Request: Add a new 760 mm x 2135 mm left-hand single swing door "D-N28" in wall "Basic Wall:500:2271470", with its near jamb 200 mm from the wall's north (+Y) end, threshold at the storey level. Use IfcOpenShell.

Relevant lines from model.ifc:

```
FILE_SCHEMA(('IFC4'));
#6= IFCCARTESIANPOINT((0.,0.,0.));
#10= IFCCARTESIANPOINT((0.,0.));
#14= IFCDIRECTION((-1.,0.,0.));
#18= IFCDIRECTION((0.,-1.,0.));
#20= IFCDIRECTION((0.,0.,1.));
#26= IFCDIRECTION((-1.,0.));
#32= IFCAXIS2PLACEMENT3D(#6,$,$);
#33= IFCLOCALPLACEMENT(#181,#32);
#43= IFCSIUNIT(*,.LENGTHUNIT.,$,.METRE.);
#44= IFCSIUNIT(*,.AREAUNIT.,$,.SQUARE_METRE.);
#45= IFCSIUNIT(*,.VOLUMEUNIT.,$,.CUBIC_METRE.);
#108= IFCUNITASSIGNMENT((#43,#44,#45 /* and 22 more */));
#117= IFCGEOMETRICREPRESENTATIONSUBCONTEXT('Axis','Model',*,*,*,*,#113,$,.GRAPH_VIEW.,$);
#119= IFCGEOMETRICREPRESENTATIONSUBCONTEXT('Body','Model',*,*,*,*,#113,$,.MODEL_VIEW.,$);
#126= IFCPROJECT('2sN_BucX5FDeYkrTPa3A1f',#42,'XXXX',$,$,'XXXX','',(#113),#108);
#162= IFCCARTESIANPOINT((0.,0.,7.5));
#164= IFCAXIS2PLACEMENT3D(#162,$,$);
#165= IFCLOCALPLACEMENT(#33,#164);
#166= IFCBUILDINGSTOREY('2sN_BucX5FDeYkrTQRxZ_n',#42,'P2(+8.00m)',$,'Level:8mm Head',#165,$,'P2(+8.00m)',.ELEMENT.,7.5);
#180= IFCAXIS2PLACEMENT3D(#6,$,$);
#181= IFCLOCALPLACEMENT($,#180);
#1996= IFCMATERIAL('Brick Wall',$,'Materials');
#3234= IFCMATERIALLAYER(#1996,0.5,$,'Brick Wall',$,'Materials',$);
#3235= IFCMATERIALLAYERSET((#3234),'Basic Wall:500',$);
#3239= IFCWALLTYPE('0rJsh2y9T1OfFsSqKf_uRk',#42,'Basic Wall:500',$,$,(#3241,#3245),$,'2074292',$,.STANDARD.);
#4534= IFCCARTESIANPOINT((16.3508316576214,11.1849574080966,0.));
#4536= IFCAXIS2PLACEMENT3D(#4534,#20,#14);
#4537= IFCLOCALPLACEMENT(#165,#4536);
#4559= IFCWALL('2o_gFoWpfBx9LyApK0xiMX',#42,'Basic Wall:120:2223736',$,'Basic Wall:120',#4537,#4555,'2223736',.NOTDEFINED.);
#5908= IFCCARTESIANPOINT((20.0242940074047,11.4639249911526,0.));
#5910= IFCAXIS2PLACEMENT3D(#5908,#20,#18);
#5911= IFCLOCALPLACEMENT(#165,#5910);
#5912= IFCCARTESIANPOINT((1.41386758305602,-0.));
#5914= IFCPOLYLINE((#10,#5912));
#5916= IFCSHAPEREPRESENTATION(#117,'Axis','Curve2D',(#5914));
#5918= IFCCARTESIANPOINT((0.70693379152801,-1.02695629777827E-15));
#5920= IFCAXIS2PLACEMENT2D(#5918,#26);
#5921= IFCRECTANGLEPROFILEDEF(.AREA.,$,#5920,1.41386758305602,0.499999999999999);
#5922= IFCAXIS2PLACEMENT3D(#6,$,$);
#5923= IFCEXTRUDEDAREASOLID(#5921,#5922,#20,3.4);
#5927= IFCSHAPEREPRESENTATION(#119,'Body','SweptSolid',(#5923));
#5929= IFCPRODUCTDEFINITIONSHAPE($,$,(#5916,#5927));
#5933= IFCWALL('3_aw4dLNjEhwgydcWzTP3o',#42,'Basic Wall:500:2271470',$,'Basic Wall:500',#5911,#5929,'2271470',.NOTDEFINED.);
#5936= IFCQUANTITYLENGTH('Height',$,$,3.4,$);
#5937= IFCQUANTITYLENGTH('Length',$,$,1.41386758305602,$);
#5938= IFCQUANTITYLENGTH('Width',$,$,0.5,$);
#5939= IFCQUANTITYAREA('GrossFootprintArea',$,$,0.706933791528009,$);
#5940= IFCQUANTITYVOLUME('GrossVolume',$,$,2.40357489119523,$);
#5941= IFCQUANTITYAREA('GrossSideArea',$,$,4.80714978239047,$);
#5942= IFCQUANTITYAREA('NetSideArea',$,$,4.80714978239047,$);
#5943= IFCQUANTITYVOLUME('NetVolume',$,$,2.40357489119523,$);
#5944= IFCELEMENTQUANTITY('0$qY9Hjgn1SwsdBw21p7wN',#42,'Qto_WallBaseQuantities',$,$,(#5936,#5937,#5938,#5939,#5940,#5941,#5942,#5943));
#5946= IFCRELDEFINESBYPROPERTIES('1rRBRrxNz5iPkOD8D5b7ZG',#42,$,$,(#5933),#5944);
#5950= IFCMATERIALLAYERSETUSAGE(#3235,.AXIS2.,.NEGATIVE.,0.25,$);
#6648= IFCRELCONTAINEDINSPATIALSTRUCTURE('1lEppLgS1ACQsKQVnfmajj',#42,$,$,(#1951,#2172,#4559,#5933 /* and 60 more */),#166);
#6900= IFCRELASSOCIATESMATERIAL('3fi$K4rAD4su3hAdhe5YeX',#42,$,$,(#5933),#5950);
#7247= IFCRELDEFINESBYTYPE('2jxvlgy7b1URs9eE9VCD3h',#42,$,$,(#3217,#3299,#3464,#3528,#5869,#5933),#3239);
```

```python
import numpy as np
import ifcopenshell
import ifcopenshell.api.feature
import ifcopenshell.api.geometry
import ifcopenshell.api.pset
import ifcopenshell.api.root
import ifcopenshell.api.spatial
import ifcopenshell.geom
import ifcopenshell.util.element
import ifcopenshell.util.placement
import ifcopenshell.util.representation
import ifcopenshell.util.shape
import ifcopenshell.util.unit

model = ifcopenshell.open("model.ifc")
unit_scale = ifcopenshell.util.unit.calculate_unit_scale(model)
area_scale = ifcopenshell.util.unit.calculate_unit_scale(model, "AREAUNIT")
volume_scale = ifcopenshell.util.unit.calculate_unit_scale(model, "VOLUMEUNIT")
settings = ifcopenshell.geom.settings()


def volume(element):
    """Net volume in cubic metres, openings subtracted."""
    shape = ifcopenshell.geom.create_shape(settings, element)
    return ifcopenshell.util.shape.get_volume(shape.geometry)


wall = model.by_guid("3_aw4dLNjEhwgydcWzTP3o")
storey = ifcopenshell.util.element.get_container(wall, ifc_class="IfcBuildingStorey")
context = ifcopenshell.util.representation.get_context(model, "Model", "Body", "MODEL_VIEW")
before = volume(wall)

width, height, from_end, sill = 0.76, 2.135, 0.2, 0.0  # metres

# The wall runs along its own X axis, and the end named is its -X end.
wall_shape = ifcopenshell.geom.create_shape(settings, wall)
x, y, z = ifcopenshell.util.shape.get_vertices(wall_shape.geometry).T
start = x.min() + from_end
face, thickness = float(y.min()), float(y.max() - y.min())
wall_matrix = ifcopenshell.util.placement.get_local_placement(wall.ObjectPlacement)
level = ifcopenshell.util.placement.get_local_placement(storey.ObjectPlacement)[2, 3]


def in_wall(x, y):
    """Placement at x, y metres in the wall's axes, at sill height."""
    matrix = wall_matrix.copy()
    matrix[:, 3] = wall_matrix @ np.array([x / unit_scale, y / unit_scale, 0.0, 1.0])
    matrix[2, 3] = level + sill / unit_scale
    return matrix


# Opening: a box that overshoots both wall faces by 50 mm.
opening = ifcopenshell.api.root.create_entity(model, ifc_class="IfcOpeningElement", predefined_type="OPENING")
box = ifcopenshell.api.geometry.add_wall_representation(
    model, context=context, length=width, height=height, thickness=thickness + 0.1
)
ifcopenshell.api.geometry.assign_representation(model, product=opening, representation=box)
ifcopenshell.api.geometry.edit_object_placement(model, product=opening, matrix=in_wall(start, face - 0.05), is_si=False)
ifcopenshell.api.feature.add_feature(model, feature=opening, element=wall)

door = ifcopenshell.api.root.create_entity(model, ifc_class="IfcDoor", name="D-N28", predefined_type="DOOR")
door.OverallWidth, door.OverallHeight = width / unit_scale, height / unit_scale
door.OperationType = "SINGLE_SWING_LEFT"
body = ifcopenshell.api.geometry.add_door_representation(
    model,
    context=context,
    overall_width=door.OverallWidth,
    overall_height=door.OverallHeight,
    operation_type="SINGLE_SWING_LEFT",
    lining_properties={"LiningDepth": thickness / unit_scale, "ThresholdDepth": thickness / unit_scale},
)
ifcopenshell.api.geometry.assign_representation(model, product=door, representation=body)
ifcopenshell.api.spatial.assign_container(model, products=[door], relating_structure=storey)
ifcopenshell.api.feature.add_filling(model, opening=opening, element=door)

# The lining spans the wall, so the door starts at the wall face.
ifcopenshell.api.geometry.edit_object_placement(model, product=door, matrix=in_wall(start, face), is_si=False)

after = volume(wall)

# Update the wall's stored quantities.
qto = model.by_id(ifcopenshell.util.element.get_pset(wall, "Qto_WallBaseQuantities", should_inherit=False)["id"])
ifcopenshell.api.pset.edit_qto(model, qto=qto, properties={
    "NetSideArea": after / thickness / area_scale,
    "NetVolume": after / volume_scale,
})

print(f"wall volume {before:.3f} -> {after:.3f} m3")

model.write("model_v2.ifc")
```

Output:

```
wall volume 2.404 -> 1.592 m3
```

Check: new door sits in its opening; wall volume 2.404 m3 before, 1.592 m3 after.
